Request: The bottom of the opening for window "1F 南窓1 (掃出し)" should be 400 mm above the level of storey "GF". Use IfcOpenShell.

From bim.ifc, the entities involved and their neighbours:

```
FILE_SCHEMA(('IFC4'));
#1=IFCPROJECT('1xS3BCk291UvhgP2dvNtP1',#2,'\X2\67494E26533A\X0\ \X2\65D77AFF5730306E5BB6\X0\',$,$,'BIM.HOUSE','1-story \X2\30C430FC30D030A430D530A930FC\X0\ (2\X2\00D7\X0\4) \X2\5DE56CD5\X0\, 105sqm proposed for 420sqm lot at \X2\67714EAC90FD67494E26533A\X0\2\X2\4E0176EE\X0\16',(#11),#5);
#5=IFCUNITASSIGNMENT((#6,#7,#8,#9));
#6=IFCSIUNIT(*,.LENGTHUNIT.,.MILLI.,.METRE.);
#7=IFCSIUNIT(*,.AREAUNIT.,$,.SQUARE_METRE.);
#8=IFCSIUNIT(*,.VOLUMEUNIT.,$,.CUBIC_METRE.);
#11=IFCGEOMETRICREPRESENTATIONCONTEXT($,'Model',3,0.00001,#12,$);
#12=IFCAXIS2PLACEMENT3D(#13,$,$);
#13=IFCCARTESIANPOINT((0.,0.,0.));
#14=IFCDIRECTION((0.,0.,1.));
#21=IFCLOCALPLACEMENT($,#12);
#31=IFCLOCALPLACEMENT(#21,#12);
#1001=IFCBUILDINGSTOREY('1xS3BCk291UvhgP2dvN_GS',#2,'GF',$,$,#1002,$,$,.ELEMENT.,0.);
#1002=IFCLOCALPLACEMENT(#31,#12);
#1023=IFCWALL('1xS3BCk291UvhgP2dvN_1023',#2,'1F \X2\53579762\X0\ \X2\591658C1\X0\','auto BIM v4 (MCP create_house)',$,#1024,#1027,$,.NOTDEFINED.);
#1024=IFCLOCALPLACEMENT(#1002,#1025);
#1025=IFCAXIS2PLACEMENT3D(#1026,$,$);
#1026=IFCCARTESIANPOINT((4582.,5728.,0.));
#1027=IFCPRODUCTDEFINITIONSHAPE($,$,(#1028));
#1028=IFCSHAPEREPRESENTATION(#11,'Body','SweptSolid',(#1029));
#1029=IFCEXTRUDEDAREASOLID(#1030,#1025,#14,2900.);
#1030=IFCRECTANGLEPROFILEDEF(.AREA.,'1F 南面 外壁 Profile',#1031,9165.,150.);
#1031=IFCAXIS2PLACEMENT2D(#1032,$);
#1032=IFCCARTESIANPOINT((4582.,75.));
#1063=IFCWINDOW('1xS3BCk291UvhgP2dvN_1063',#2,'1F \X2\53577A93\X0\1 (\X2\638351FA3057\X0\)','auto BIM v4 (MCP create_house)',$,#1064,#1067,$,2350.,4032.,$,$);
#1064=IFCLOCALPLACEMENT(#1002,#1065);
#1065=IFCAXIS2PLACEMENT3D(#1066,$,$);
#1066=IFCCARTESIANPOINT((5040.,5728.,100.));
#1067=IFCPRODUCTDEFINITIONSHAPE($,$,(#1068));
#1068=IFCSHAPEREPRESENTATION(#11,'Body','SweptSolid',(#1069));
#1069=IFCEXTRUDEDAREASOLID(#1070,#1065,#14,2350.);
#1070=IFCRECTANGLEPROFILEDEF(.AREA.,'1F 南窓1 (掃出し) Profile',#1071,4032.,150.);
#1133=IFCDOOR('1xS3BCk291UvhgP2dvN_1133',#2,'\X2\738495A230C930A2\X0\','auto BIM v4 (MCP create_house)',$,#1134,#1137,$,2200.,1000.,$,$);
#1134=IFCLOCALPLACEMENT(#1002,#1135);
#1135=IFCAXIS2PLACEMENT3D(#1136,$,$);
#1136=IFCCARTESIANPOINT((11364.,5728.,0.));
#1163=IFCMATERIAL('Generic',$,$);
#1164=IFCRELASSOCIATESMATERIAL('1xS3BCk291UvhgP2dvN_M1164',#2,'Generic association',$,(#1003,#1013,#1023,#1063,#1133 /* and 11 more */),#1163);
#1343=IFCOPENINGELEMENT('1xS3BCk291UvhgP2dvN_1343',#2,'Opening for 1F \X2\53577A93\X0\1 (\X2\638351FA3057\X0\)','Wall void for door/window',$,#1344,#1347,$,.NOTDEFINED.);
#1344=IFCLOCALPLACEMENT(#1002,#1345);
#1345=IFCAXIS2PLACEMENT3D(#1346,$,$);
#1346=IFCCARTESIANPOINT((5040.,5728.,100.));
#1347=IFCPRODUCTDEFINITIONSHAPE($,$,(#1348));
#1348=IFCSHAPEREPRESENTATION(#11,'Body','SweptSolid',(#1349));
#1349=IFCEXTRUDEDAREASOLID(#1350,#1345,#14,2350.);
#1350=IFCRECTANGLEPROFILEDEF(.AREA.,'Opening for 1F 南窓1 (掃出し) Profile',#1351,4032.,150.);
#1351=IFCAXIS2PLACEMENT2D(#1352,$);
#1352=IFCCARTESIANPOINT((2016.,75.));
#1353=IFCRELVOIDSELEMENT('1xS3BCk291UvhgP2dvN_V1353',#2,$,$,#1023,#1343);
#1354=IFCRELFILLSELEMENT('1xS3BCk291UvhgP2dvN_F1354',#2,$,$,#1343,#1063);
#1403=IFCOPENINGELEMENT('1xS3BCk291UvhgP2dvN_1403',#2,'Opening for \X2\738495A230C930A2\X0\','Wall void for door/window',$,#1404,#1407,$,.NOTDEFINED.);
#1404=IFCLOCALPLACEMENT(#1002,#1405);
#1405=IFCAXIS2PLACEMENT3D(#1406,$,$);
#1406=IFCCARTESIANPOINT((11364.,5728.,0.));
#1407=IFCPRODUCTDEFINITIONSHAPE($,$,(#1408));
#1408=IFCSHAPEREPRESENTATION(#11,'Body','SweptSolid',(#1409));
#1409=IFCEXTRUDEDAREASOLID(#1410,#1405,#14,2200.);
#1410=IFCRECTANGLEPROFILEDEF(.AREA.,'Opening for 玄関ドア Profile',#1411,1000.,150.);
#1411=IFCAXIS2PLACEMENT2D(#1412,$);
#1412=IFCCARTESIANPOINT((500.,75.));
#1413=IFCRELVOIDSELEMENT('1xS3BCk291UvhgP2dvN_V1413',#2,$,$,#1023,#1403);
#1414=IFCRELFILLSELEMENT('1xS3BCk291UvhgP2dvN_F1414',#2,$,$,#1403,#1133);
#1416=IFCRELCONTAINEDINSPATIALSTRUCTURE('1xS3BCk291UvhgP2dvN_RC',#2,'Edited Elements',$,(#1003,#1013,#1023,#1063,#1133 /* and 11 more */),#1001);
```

```python
import numpy as np
import ifcopenshell
import ifcopenshell.api.geometry
import ifcopenshell.geom
import ifcopenshell.util.element
import ifcopenshell.util.placement
import ifcopenshell.util.shape
import ifcopenshell.util.unit

model = ifcopenshell.open("bim.ifc")
unit_scale = ifcopenshell.util.unit.calculate_unit_scale(model)

window = model.by_guid("1xS3BCk291UvhgP2dvN_1063")
opening = window.FillsVoids[0].RelatingOpeningElement
storey = ifcopenshell.util.element.get_container(window, ifc_class="IfcBuildingStorey")
level = ifcopenshell.util.placement.get_local_placement(storey.ObjectPlacement)[2, 3]

# The opening's origin need not be at the sill, so measure its lowest point.
shape = ifcopenshell.geom.create_shape(ifcopenshell.geom.settings(), opening)
bottom = ifcopenshell.util.shape.get_shape_bottom_elevation(shape, shape.geometry) / unit_scale
dz = level + 0.4 / unit_scale - bottom

shift = np.array([0.0, 0.0, dz])
# The window is not placed relative to its opening, so move both.
for product in (opening, window):
    matrix = ifcopenshell.util.placement.get_local_placement(product.ObjectPlacement)
    matrix[:3, 3] += shift
    ifcopenshell.api.geometry.edit_object_placement(model, product=product, matrix=matrix, is_si=False)

print(f"moved by {dz * unit_scale:+.3f} m")

model.write("bim-out.ifc")
```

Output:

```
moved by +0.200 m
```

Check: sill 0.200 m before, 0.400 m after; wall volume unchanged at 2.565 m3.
